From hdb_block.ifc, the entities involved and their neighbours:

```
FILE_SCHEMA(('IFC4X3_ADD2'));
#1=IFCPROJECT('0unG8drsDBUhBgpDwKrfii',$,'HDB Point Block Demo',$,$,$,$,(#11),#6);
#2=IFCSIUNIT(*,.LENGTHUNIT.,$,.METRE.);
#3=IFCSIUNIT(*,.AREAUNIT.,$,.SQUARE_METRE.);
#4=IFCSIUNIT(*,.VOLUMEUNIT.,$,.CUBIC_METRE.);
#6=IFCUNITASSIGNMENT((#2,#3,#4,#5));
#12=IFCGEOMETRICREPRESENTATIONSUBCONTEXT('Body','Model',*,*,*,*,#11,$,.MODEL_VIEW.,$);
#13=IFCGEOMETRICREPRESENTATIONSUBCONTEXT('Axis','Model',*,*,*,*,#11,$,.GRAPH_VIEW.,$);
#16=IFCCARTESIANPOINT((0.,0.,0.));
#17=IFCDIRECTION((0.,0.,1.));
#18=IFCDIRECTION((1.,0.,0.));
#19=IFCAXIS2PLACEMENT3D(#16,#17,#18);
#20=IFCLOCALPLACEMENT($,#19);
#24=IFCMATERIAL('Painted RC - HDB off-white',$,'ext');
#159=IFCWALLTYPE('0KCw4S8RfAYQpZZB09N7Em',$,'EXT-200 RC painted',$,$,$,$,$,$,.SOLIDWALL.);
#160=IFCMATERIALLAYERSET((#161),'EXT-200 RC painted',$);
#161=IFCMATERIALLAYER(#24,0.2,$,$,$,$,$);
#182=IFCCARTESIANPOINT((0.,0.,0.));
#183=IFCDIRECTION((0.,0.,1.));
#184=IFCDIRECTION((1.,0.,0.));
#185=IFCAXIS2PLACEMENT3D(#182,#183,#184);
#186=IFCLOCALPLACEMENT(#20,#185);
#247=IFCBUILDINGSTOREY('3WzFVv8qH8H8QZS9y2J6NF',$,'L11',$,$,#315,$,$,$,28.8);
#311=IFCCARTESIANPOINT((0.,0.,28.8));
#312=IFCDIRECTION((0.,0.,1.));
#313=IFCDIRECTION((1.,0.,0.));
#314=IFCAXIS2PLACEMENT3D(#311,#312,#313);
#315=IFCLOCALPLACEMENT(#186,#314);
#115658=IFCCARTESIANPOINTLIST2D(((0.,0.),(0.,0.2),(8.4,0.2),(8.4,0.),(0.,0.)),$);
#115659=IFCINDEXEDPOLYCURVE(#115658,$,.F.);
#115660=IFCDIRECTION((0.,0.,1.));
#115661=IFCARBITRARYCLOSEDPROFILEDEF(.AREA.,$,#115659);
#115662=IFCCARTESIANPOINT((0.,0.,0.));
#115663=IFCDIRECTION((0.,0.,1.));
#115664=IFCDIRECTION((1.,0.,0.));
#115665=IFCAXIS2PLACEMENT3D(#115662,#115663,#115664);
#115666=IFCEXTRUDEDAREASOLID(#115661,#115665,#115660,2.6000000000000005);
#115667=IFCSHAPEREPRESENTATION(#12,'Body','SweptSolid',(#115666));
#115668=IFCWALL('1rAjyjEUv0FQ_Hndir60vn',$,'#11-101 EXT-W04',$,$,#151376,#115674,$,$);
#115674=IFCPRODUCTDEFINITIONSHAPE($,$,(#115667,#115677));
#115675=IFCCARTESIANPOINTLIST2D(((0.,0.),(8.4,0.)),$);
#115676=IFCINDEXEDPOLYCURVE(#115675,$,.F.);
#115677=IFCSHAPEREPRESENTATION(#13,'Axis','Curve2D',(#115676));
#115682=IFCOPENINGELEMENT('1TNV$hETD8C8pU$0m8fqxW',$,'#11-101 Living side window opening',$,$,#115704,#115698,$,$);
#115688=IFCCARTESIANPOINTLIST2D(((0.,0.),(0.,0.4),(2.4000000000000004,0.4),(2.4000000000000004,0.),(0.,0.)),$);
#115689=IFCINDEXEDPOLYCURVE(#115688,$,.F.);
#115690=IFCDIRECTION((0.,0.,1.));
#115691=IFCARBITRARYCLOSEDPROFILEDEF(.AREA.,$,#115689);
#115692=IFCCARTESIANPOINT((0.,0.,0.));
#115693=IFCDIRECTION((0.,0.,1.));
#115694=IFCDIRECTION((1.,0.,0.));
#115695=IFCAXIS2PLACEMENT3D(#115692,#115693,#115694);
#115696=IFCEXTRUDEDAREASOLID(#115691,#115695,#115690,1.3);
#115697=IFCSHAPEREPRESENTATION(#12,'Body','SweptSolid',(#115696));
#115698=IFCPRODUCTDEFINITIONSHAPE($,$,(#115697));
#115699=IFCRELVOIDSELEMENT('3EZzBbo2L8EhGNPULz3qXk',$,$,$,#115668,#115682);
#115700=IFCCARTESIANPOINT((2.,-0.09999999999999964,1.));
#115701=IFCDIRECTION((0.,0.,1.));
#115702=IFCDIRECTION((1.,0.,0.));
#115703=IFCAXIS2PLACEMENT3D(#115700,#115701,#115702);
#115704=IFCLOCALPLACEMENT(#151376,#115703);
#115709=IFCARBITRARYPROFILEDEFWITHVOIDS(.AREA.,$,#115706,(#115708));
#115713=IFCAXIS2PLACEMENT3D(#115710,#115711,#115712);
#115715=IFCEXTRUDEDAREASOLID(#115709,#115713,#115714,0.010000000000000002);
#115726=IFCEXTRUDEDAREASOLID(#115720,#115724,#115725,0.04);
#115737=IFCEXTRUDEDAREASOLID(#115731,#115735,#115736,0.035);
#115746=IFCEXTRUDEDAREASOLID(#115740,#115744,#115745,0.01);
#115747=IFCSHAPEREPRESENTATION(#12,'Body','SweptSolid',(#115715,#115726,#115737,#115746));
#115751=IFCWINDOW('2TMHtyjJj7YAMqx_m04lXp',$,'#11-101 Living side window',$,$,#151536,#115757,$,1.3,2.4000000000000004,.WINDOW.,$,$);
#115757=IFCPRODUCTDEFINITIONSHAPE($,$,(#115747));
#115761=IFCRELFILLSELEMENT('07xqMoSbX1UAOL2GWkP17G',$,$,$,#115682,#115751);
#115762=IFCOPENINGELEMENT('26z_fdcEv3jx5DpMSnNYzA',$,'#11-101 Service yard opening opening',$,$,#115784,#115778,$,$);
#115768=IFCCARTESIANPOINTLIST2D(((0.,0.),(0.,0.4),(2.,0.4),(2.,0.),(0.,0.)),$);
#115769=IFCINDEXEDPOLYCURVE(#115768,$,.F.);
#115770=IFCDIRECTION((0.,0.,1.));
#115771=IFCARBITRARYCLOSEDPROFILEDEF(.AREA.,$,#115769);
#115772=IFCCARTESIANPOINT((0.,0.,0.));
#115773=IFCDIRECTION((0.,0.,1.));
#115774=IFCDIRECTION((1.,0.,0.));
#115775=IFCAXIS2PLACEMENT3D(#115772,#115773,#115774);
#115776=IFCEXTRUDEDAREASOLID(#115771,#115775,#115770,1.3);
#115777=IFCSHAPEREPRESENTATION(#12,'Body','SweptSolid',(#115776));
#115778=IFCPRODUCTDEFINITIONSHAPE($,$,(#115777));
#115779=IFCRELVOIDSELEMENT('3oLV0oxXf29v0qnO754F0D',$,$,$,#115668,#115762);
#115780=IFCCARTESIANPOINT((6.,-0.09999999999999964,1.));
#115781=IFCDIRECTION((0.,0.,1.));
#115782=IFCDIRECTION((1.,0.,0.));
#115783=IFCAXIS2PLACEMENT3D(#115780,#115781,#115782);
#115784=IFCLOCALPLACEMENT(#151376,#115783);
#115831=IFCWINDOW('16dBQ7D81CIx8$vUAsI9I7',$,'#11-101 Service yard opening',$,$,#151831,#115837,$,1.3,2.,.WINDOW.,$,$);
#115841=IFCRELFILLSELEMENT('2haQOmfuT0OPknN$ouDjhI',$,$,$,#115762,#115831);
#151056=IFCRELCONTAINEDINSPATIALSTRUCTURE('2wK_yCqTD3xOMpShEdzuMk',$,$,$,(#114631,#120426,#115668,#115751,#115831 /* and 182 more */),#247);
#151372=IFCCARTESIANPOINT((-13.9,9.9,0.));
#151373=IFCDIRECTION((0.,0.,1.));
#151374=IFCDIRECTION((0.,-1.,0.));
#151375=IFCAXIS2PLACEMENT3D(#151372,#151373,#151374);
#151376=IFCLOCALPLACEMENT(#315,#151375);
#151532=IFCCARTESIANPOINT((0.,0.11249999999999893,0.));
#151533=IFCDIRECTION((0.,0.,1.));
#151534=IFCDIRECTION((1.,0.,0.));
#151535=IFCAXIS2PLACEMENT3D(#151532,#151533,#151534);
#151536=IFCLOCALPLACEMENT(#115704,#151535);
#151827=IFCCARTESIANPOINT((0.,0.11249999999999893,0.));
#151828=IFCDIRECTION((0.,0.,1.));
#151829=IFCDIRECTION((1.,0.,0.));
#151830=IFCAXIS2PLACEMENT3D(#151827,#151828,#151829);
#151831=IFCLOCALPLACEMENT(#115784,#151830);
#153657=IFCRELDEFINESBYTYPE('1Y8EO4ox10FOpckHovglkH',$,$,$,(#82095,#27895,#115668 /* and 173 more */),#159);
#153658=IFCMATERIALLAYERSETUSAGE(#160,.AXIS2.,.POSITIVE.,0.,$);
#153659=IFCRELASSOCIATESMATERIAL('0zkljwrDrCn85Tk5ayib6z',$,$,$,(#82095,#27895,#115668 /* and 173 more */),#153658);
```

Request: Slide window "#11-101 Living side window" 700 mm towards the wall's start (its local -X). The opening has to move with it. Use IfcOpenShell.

```python
import ifcopenshell
import ifcopenshell.api.geometry
import ifcopenshell.util.placement

model = ifcopenshell.open("hdb_block.ifc")

window = model.by_id(115751)
opening = window.FillsVoids[0].RelatingOpeningElement
wall = opening.VoidsElements[0].RelatingBuildingElement

wall_matrix = ifcopenshell.util.placement.get_local_placement(wall.ObjectPlacement)
shift = wall_matrix[:3, 0] * -0.7
before = ifcopenshell.util.placement.get_local_placement(window.ObjectPlacement)[:3, 3].copy()

# The window is placed relative to its opening, so it follows when the opening moves.
matrix = ifcopenshell.util.placement.get_local_placement(opening.ObjectPlacement)
matrix[:3, 3] += shift
ifcopenshell.api.geometry.edit_object_placement(
    model, product=opening, matrix=matrix, is_si=False, should_transform_children=True
)

after = ifcopenshell.util.placement.get_local_placement(window.ObjectPlacement)[:3, 3]
print("window moved by", (after - before).round(3) + 0.0)

model.write("hdb_block-out.ifc")
```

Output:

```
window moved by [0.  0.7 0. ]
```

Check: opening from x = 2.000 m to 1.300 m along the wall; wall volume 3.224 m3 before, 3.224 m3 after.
